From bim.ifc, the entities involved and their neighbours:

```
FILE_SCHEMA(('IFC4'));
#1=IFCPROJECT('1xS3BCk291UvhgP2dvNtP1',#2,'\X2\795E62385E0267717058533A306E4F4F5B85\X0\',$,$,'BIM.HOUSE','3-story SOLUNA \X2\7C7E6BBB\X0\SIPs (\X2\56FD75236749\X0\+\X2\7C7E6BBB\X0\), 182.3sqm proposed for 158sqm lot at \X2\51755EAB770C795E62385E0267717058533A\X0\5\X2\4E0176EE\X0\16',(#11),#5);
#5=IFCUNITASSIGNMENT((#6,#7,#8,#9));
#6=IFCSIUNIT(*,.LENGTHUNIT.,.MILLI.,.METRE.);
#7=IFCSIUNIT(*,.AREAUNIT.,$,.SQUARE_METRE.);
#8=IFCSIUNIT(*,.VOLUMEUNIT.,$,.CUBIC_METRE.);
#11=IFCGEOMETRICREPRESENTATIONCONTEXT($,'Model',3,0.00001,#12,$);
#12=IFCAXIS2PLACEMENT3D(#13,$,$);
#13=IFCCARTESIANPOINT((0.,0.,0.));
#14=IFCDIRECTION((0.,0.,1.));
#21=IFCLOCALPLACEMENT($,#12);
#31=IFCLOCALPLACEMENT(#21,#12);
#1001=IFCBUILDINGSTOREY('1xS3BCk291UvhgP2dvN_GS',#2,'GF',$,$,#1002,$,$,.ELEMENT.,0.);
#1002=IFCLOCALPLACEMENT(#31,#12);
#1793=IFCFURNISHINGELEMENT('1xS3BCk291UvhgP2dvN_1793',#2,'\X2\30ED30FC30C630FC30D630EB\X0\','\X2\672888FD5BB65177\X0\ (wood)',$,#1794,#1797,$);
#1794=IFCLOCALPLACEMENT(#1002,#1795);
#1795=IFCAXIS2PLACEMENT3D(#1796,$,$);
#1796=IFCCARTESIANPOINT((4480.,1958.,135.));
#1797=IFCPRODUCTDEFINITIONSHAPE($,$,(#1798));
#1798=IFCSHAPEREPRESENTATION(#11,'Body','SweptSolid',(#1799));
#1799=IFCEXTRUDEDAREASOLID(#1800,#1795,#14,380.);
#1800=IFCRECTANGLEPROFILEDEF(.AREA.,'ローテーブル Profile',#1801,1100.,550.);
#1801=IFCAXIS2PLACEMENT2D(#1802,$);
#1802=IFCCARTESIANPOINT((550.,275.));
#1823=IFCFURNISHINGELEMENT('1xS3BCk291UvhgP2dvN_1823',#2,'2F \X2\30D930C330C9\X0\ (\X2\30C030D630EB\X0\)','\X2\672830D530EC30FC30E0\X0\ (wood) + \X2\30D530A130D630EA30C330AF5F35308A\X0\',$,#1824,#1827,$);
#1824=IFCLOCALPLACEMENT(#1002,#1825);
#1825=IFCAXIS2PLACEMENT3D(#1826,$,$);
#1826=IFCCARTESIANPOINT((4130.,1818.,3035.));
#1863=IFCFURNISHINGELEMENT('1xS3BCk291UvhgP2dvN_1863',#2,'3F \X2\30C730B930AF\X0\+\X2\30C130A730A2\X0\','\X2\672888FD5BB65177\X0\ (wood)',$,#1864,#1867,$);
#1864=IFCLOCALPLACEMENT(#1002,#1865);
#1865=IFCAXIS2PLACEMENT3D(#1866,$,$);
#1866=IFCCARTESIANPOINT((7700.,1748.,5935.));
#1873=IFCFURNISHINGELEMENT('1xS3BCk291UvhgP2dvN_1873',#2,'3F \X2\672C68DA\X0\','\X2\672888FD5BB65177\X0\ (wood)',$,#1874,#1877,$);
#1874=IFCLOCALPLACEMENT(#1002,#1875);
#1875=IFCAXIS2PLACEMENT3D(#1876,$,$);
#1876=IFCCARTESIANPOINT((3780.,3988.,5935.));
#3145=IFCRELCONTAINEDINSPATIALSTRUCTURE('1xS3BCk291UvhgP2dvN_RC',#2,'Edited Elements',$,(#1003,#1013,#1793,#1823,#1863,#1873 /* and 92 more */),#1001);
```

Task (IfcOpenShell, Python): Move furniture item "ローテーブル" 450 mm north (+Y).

```python
import ifcopenshell
import ifcopenshell.api.geometry
import ifcopenshell.util.placement

model = ifcopenshell.open("bim.ifc")

item = model.by_guid("1xS3BCk291UvhgP2dvN_1793")
matrix = ifcopenshell.util.placement.get_local_placement(item.ObjectPlacement)
matrix[1, 3] += 450.0
ifcopenshell.api.geometry.edit_object_placement(model, product=item, matrix=matrix, is_si=False)

print(ifcopenshell.util.placement.get_local_placement(item.ObjectPlacement).round(3) + 0.0)

model.write("bim_v2.ifc")
```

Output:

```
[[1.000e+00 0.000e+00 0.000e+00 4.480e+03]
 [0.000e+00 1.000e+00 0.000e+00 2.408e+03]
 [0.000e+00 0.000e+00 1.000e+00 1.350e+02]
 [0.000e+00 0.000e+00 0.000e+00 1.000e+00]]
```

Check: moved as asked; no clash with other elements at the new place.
